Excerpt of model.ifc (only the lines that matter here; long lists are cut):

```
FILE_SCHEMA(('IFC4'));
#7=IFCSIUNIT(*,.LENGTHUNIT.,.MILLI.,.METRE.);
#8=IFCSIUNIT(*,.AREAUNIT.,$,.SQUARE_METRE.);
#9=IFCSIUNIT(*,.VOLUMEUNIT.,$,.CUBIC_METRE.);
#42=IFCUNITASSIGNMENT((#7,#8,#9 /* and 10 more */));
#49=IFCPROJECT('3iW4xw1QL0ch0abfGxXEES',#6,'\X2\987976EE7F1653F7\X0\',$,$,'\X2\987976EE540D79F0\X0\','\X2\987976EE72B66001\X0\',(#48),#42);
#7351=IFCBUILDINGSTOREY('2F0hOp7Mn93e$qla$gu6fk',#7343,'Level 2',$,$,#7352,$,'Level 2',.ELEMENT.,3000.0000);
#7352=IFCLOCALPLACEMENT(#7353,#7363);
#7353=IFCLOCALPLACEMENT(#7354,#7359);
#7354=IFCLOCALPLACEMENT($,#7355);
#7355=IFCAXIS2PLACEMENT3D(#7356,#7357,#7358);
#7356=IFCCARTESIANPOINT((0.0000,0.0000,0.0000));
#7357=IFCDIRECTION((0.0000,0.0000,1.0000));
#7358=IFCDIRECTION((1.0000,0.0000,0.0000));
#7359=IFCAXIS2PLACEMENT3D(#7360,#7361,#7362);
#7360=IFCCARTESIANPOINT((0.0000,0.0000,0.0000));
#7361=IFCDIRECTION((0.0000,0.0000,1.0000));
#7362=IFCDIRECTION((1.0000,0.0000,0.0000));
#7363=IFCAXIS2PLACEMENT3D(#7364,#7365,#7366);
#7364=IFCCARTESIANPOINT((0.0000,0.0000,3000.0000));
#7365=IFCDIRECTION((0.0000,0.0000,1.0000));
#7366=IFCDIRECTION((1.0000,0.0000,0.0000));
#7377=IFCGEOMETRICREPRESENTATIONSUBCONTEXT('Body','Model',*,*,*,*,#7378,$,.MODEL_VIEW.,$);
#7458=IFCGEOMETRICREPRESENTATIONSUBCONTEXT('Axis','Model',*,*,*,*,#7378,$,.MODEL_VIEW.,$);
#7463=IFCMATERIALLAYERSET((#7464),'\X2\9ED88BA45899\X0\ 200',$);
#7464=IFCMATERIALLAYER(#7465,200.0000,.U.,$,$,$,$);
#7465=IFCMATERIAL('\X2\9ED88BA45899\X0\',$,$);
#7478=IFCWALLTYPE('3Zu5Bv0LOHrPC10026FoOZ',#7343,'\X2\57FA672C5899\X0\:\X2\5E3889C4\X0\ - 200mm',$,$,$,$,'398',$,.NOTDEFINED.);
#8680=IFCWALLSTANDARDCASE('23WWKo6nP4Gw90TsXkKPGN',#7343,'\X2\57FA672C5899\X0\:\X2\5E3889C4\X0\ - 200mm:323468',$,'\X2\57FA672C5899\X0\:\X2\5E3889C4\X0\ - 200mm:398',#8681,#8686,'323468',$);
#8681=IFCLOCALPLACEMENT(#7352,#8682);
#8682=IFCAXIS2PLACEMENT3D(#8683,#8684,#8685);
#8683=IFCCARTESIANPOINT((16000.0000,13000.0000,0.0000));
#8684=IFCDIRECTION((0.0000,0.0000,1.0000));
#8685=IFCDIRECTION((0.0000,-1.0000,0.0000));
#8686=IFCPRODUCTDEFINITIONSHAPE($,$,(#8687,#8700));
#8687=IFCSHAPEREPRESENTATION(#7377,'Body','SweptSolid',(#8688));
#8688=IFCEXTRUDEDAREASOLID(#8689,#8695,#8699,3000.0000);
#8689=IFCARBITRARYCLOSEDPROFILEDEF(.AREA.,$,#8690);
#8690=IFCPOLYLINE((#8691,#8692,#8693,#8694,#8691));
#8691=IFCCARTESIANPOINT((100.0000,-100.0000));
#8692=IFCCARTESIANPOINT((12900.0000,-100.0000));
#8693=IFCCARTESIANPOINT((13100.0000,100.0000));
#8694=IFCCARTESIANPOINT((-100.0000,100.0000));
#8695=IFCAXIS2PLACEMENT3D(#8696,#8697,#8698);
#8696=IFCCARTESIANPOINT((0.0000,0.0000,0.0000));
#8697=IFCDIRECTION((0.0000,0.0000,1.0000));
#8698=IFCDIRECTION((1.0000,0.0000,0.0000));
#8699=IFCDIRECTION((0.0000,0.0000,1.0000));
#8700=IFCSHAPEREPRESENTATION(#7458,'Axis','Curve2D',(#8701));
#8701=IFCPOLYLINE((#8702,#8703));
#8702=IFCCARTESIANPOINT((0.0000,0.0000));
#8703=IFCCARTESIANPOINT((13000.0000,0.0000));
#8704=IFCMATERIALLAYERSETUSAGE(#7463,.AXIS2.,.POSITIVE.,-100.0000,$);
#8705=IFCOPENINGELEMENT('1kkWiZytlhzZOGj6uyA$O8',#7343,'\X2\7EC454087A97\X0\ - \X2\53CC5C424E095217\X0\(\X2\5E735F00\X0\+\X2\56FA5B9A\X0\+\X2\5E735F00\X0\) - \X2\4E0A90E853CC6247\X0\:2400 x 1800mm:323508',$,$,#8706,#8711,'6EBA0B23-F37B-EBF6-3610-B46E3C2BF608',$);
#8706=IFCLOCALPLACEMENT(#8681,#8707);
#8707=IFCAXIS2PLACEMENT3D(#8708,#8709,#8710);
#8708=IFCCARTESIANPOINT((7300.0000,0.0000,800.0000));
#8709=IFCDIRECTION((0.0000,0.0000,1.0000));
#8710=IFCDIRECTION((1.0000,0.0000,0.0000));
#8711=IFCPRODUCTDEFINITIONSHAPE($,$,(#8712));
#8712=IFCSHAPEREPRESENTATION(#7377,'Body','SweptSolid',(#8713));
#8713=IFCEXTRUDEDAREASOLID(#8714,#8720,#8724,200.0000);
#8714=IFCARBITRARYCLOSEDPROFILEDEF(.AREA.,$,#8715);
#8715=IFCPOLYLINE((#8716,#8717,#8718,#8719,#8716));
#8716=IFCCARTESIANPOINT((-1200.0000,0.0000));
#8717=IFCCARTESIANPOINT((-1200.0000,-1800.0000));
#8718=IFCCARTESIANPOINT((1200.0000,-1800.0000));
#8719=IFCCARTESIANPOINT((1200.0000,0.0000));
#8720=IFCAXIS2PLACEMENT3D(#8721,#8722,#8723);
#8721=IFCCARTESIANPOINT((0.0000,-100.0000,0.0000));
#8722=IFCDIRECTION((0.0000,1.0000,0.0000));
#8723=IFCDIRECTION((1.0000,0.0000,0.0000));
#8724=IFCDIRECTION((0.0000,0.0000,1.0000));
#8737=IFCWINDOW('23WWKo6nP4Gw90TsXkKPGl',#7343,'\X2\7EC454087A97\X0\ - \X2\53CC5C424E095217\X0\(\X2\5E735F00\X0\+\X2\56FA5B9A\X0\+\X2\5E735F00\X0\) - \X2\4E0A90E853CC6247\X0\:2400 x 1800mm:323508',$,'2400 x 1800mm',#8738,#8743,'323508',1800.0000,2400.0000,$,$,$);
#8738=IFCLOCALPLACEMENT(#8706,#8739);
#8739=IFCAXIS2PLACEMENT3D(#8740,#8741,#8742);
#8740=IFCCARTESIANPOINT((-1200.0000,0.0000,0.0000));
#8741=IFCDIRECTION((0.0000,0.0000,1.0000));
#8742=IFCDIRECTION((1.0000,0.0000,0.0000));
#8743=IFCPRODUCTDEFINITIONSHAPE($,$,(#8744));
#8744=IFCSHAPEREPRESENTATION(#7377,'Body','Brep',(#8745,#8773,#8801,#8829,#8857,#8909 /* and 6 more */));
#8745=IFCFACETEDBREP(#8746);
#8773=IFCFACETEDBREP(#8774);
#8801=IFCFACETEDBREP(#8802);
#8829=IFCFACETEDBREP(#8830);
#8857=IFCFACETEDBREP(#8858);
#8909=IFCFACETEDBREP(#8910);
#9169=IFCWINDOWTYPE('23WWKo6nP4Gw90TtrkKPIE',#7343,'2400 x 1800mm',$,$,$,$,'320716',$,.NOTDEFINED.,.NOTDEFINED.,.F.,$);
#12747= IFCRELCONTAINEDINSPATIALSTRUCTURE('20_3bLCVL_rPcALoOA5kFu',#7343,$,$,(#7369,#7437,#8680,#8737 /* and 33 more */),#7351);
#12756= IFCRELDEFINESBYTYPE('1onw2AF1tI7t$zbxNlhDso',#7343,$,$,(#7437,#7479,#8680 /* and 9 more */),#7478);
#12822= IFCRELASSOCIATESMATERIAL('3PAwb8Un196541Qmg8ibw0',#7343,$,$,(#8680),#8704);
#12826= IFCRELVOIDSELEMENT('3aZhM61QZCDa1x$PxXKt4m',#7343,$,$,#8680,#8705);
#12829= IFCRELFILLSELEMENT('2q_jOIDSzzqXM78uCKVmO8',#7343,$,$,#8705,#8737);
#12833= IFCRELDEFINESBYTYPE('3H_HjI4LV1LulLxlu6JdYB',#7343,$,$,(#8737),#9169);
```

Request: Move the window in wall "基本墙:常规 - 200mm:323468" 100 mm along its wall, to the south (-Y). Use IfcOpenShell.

```python
import ifcopenshell
import ifcopenshell.api.geometry
import ifcopenshell.util.placement
import ifcopenshell.util.unit

model = ifcopenshell.open("model.ifc")
unit_scale = ifcopenshell.util.unit.calculate_unit_scale(model)

window = model.by_id(8737)
opening = window.FillsVoids[0].RelatingOpeningElement
wall = opening.VoidsElements[0].RelatingBuildingElement

wall_matrix = ifcopenshell.util.placement.get_local_placement(wall.ObjectPlacement)
shift = wall_matrix[:3, 0] * 0.1 / unit_scale
before = ifcopenshell.util.placement.get_local_placement(window.ObjectPlacement)[:3, 3].copy()

# The window is placed relative to its opening, so it follows when the opening moves.
matrix = ifcopenshell.util.placement.get_local_placement(opening.ObjectPlacement)
matrix[:3, 3] += shift
ifcopenshell.api.geometry.edit_object_placement(
    model, product=opening, matrix=matrix, is_si=False, should_transform_children=True
)

after = ifcopenshell.util.placement.get_local_placement(window.ObjectPlacement)[:3, 3]
print("window moved by", (after - before).round(3) + 0.0)

model.write("model_v2.ifc")
```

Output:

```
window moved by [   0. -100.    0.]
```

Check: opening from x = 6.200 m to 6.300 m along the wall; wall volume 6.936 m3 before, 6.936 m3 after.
